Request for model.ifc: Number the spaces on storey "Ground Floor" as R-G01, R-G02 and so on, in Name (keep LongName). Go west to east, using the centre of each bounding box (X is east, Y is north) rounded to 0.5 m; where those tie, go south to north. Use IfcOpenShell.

First a look at what the model holds.

```python
import ifcopenshell
import ifcopenshell.util.element
import ifcopenshell.util.placement

model = ifcopenshell.open("model.ifc")
print(model.schema)
storey = next(s for s in model.by_type("IfcBuildingStorey") if s.Name == "Ground Floor")
spaces = [e for e in ifcopenshell.util.element.get_decomposition(storey) if e.is_a("IfcSpace")]
for e in sorted(spaces, key=lambda e: e.id()):
    origin = ifcopenshell.util.placement.get_local_placement(e.ObjectPlacement)[:3, 3]
    print(e.id(), e.Name, e.LongName, origin.round(2) + 0.0, sep=" | ")
```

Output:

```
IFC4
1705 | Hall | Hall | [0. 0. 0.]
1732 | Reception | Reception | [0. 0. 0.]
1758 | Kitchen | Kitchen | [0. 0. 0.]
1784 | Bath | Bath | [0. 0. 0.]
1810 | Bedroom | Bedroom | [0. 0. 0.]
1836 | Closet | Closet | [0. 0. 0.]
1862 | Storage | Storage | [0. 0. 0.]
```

```python
import ifcopenshell
import ifcopenshell.geom
import ifcopenshell.util.element
import ifcopenshell.util.shape

model = ifcopenshell.open("model.ifc")
settings = ifcopenshell.geom.settings()
settings.set("use-world-coords", True)


def centre(element):
    shape = ifcopenshell.geom.create_shape(settings, element)
    return ifcopenshell.util.shape.get_bbox_centroid(shape.geometry)


storey = next(s for s in model.by_type("IfcBuildingStorey") if s.Name == "Ground Floor")
spaces = [e for e in ifcopenshell.util.element.get_decomposition(storey) if e.is_a("IfcSpace")]

# Insertion points can sit at a corner or the storey origin, so sort by the geometry (in metres).
centres = {e: centre(e) for e in spaces}
spaces.sort(key=lambda e: (round(centres[e][0] / 0.5), centres[e][1]))

for i, e in enumerate(spaces, start=1):
    number = f"R-G{i:02d}"
    e.Name = number
    print(e.id(), number)

model.write("model_v2.ifc")
```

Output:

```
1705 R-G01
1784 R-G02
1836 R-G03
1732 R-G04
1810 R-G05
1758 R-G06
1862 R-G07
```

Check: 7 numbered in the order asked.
